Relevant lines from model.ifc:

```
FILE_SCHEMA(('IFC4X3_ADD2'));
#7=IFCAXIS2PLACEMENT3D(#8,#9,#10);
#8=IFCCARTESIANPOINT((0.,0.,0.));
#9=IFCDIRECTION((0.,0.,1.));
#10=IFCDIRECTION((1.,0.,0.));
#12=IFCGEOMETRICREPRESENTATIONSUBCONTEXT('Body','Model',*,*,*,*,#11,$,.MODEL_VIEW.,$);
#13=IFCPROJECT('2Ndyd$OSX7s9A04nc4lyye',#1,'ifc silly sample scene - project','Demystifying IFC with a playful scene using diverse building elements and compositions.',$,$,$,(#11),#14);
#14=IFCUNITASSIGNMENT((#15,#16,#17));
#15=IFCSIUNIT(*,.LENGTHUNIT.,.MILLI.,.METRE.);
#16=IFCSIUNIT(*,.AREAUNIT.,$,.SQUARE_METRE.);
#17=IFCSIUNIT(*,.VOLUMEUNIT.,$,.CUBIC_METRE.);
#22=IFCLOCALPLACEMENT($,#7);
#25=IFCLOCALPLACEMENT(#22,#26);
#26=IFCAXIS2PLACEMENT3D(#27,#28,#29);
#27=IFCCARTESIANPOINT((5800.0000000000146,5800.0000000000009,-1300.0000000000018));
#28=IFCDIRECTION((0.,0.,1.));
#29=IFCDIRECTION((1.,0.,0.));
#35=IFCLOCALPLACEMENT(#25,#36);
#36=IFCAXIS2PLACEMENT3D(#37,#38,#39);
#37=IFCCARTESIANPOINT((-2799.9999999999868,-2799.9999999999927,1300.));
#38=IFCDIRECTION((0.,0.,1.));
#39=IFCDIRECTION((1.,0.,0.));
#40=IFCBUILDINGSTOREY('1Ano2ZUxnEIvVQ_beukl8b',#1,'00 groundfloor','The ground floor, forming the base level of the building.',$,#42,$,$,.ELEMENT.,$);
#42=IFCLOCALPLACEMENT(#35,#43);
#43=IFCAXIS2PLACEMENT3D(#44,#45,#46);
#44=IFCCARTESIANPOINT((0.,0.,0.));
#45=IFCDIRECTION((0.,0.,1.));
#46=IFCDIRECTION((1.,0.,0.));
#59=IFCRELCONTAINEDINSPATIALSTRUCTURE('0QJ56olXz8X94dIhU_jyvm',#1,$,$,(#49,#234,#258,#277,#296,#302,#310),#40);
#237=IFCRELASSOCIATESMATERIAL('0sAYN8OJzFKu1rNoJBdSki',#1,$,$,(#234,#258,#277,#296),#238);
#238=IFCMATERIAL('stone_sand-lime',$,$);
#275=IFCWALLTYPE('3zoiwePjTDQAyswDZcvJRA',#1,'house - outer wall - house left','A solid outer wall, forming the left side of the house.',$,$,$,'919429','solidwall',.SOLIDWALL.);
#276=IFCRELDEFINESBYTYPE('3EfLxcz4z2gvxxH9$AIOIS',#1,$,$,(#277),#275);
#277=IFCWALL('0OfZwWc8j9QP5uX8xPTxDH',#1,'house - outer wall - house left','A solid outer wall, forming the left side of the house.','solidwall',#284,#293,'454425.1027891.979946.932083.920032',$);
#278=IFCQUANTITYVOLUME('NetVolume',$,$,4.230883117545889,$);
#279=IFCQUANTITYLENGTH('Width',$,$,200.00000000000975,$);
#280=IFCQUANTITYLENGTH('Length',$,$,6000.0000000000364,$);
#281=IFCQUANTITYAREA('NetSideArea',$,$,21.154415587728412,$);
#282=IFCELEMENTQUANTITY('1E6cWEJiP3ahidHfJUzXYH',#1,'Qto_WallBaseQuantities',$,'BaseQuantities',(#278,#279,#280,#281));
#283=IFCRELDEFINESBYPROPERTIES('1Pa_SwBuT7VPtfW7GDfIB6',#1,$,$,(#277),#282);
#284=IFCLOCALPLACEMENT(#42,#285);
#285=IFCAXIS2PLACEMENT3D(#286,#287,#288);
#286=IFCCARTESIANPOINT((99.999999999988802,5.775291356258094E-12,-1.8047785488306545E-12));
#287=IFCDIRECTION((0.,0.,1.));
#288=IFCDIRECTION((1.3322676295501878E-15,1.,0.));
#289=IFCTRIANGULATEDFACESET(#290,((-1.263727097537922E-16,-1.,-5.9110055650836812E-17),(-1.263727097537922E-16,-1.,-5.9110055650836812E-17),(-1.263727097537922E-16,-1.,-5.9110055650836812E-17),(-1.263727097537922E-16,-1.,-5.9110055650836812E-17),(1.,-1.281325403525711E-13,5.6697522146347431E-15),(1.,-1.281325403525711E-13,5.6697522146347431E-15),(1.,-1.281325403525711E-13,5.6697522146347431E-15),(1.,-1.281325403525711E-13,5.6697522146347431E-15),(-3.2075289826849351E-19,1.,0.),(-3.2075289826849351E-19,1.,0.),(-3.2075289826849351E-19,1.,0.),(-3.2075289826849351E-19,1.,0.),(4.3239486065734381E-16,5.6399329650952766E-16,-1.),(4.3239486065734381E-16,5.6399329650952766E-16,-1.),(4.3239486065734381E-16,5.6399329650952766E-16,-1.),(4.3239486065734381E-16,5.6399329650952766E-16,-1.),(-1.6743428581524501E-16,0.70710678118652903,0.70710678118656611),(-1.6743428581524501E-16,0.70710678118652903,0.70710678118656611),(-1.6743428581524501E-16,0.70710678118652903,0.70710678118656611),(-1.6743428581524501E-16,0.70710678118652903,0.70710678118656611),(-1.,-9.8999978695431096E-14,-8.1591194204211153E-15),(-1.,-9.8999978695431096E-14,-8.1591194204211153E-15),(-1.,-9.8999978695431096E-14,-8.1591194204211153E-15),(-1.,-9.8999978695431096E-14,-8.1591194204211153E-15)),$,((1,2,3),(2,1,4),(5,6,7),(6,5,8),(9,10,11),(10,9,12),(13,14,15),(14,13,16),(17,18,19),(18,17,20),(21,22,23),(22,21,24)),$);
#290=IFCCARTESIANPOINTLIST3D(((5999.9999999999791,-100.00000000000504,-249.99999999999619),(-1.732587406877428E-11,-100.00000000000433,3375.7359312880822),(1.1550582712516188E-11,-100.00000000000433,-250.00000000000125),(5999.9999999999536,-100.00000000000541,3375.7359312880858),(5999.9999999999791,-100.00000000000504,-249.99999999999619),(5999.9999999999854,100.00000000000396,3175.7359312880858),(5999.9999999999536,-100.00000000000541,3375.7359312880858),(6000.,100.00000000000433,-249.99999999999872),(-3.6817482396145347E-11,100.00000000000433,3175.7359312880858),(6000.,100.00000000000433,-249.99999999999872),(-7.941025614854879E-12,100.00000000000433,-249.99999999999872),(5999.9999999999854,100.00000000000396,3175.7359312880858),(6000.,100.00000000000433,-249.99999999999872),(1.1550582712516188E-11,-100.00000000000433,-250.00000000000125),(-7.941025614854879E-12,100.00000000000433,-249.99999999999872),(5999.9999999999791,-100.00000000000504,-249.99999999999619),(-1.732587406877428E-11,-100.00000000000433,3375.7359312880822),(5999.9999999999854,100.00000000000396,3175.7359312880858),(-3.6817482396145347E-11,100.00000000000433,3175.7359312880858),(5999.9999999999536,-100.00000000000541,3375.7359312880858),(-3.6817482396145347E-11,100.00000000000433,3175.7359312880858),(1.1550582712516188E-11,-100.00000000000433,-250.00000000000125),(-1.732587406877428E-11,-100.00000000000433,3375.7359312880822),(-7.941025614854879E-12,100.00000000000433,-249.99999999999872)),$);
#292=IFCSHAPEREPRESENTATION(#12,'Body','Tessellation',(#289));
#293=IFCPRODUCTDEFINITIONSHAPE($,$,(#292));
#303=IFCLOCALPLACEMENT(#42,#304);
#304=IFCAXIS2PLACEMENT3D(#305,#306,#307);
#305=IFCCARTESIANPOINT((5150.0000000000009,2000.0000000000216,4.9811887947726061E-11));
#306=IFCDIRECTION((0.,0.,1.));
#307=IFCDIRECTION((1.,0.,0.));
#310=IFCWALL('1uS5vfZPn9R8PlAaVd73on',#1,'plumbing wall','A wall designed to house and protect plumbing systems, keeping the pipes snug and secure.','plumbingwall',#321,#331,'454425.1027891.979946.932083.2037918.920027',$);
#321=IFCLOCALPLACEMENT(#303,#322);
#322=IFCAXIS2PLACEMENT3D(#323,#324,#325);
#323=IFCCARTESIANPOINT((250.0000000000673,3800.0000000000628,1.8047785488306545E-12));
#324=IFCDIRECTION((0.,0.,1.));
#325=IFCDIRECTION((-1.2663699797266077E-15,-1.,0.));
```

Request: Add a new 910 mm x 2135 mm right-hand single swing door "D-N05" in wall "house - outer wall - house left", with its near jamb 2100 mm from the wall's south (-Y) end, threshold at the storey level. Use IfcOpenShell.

```python
import numpy as np
import ifcopenshell
import ifcopenshell.api.feature
import ifcopenshell.api.geometry
import ifcopenshell.api.pset
import ifcopenshell.api.root
import ifcopenshell.api.spatial
import ifcopenshell.geom
import ifcopenshell.util.element
import ifcopenshell.util.placement
import ifcopenshell.util.representation
import ifcopenshell.util.shape
import ifcopenshell.util.unit

model = ifcopenshell.open("model.ifc")
unit_scale = ifcopenshell.util.unit.calculate_unit_scale(model)
area_scale = ifcopenshell.util.unit.calculate_unit_scale(model, "AREAUNIT")
volume_scale = ifcopenshell.util.unit.calculate_unit_scale(model, "VOLUMEUNIT")
settings = ifcopenshell.geom.settings()


def volume(element):
    """Net volume in cubic metres, openings subtracted."""
    shape = ifcopenshell.geom.create_shape(settings, element)
    return ifcopenshell.util.shape.get_volume(shape.geometry)


wall = model.by_id(277)
storey = ifcopenshell.util.element.get_container(wall, ifc_class="IfcBuildingStorey")
context = ifcopenshell.util.representation.get_context(model, "Model", "Body", "MODEL_VIEW")
before = volume(wall)

width, height, from_end, sill = 0.91, 2.135, 2.1, 0.0  # metres

# The wall runs along its own X axis, and the end named is its -X end.
wall_shape = ifcopenshell.geom.create_shape(settings, wall)
x, y, z = ifcopenshell.util.shape.get_vertices(wall_shape.geometry).T
start = x.min() + from_end
face, thickness = float(y.min()), float(y.max() - y.min())
wall_matrix = ifcopenshell.util.placement.get_local_placement(wall.ObjectPlacement)
level = ifcopenshell.util.placement.get_local_placement(storey.ObjectPlacement)[2, 3]


def in_wall(x, y):
    """Placement at x, y metres in the wall's axes, at sill height."""
    matrix = wall_matrix.copy()
    matrix[:, 3] = wall_matrix @ np.array([x / unit_scale, y / unit_scale, 0.0, 1.0])
    matrix[2, 3] = level + sill / unit_scale
    return matrix


# Opening: a box that overshoots both wall faces by 50 mm.
opening = ifcopenshell.api.root.create_entity(model, ifc_class="IfcOpeningElement", predefined_type="OPENING")
box = ifcopenshell.api.geometry.add_wall_representation(
    model, context=context, length=width, height=height, thickness=thickness + 0.1
)
ifcopenshell.api.geometry.assign_representation(model, product=opening, representation=box)
ifcopenshell.api.geometry.edit_object_placement(model, product=opening, matrix=in_wall(start, face - 0.05), is_si=False)
ifcopenshell.api.feature.add_feature(model, feature=opening, element=wall)

door = ifcopenshell.api.root.create_entity(model, ifc_class="IfcDoor", name="D-N05", predefined_type="DOOR")
door.OverallWidth, door.OverallHeight = width / unit_scale, height / unit_scale
door.OperationType = "SINGLE_SWING_RIGHT"
body = ifcopenshell.api.geometry.add_door_representation(
    model,
    context=context,
    overall_width=door.OverallWidth,
    overall_height=door.OverallHeight,
    operation_type="SINGLE_SWING_RIGHT",
    lining_properties={"LiningDepth": thickness / unit_scale, "ThresholdDepth": thickness / unit_scale},
)
ifcopenshell.api.geometry.assign_representation(model, product=door, representation=body)
ifcopenshell.api.spatial.assign_container(model, products=[door], relating_structure=storey)
ifcopenshell.api.feature.add_filling(model, opening=opening, element=door)

# The lining spans the wall, so the door starts at the wall face.
ifcopenshell.api.geometry.edit_object_placement(model, product=door, matrix=in_wall(start, face), is_si=False)

after = volume(wall)

# Update the wall's stored quantities.
qto = model.by_id(ifcopenshell.util.element.get_pset(wall, "Qto_WallBaseQuantities", should_inherit=False)["id"])
ifcopenshell.api.pset.edit_qto(model, qto=qto, properties={
    "NetVolume": after / volume_scale,
    "NetSideArea": after / thickness / area_scale,
})

print(f"wall volume {before:.3f} -> {after:.3f} m3")

model.write("model_rev.ifc")
```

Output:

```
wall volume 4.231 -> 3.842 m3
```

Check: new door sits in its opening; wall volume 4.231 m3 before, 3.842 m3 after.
